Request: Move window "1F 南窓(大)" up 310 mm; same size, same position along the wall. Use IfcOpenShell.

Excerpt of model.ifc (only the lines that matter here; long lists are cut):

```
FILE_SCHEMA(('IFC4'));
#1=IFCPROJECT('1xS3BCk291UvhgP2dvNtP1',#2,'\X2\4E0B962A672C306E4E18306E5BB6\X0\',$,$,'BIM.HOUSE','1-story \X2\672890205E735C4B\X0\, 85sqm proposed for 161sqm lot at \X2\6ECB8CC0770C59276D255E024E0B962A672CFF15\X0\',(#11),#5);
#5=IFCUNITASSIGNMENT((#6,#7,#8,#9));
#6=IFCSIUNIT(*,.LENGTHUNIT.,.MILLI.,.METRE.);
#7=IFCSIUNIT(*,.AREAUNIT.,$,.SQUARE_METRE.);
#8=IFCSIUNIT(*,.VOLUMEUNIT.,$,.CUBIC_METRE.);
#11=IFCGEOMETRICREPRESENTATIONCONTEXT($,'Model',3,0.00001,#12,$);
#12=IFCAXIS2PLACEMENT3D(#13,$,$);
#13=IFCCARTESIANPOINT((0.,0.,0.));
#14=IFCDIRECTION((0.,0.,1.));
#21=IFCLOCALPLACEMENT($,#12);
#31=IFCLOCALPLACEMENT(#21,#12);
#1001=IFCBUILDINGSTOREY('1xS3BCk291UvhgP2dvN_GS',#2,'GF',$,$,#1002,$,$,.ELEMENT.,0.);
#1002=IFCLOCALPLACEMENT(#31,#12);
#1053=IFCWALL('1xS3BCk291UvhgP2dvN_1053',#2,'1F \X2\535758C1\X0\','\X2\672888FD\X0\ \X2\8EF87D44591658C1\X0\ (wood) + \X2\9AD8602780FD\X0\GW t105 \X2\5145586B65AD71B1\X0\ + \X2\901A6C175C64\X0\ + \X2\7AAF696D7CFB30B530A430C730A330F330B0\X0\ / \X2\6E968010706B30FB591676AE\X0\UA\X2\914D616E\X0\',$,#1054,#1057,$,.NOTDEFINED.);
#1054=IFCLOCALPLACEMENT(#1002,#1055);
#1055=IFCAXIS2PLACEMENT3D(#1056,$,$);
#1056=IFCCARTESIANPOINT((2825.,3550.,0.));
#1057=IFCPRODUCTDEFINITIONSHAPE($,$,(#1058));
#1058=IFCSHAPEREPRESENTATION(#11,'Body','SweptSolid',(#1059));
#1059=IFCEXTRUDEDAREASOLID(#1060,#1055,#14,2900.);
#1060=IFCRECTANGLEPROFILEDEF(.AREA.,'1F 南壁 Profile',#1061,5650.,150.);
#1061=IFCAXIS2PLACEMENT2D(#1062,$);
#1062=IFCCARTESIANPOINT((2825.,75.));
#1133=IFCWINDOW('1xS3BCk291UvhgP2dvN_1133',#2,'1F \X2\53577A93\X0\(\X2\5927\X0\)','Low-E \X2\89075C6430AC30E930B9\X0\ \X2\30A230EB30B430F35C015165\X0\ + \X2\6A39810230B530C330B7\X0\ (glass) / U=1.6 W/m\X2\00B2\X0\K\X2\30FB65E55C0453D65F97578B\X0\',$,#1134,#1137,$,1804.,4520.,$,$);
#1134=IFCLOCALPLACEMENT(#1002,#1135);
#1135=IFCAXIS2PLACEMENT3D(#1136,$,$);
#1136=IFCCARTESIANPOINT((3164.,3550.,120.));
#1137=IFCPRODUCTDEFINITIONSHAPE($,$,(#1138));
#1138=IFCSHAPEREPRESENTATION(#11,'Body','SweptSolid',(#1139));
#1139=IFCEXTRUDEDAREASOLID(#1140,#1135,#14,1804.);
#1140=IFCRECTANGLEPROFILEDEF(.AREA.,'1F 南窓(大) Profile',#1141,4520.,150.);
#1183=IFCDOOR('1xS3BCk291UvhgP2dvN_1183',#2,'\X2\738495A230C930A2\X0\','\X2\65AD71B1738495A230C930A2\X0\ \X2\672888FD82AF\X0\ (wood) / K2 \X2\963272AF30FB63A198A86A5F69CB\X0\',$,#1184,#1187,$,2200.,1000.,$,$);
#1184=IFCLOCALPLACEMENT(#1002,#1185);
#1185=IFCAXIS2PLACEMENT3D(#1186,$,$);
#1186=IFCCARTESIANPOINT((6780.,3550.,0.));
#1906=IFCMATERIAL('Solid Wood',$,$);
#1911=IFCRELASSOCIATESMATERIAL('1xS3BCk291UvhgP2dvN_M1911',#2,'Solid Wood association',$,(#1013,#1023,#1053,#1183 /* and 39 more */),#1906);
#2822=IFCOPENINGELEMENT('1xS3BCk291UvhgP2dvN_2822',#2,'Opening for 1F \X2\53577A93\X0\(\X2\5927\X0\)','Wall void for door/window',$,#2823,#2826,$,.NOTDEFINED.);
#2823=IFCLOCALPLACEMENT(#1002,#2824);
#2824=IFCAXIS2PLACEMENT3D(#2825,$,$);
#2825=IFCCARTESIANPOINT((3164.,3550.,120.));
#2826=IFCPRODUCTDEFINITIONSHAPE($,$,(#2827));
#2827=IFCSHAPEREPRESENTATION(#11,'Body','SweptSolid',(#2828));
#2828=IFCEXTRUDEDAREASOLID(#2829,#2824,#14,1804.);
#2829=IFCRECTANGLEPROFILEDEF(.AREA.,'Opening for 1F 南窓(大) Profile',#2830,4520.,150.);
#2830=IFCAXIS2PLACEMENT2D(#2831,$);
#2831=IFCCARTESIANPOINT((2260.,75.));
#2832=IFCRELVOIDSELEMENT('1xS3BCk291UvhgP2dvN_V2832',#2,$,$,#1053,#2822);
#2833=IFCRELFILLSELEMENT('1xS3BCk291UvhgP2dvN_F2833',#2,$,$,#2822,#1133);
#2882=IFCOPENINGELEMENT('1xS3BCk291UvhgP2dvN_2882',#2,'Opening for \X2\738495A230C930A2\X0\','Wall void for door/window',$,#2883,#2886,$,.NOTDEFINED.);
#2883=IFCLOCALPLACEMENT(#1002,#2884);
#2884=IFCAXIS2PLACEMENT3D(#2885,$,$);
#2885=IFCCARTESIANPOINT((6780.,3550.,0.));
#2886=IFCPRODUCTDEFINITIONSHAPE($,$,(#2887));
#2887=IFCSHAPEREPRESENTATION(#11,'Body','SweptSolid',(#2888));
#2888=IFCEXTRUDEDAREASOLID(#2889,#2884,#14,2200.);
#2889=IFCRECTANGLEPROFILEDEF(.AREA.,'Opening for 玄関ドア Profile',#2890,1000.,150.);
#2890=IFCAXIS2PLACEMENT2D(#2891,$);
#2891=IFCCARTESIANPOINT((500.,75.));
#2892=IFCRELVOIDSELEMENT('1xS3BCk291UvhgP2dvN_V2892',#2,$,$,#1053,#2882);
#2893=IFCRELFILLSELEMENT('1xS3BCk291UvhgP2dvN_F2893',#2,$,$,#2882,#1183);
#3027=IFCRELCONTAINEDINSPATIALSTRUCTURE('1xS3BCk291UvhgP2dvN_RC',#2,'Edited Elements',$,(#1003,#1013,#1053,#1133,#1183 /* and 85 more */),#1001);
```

```python
import numpy as np
import ifcopenshell
import ifcopenshell.api.geometry
import ifcopenshell.util.placement
import ifcopenshell.util.unit

model = ifcopenshell.open("model.ifc")
unit_scale = ifcopenshell.util.unit.calculate_unit_scale(model)

window = model.by_guid("1xS3BCk291UvhgP2dvN_1133")
opening = window.FillsVoids[0].RelatingOpeningElement
dz = 0.31 / unit_scale

shift = np.array([0.0, 0.0, dz])
# The window is not placed relative to its opening, so move both.
for product in (opening, window):
    matrix = ifcopenshell.util.placement.get_local_placement(product.ObjectPlacement)
    matrix[:3, 3] += shift
    ifcopenshell.api.geometry.edit_object_placement(model, product=product, matrix=matrix, is_si=False)

print(f"moved by {dz * unit_scale:+.3f} m")

model.write("model_updated.ifc")
```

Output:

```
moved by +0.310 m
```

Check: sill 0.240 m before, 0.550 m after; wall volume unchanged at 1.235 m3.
